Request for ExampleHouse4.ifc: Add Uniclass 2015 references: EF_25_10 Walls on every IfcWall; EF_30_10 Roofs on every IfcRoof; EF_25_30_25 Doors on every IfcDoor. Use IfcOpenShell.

First a look at what the model holds.

```python
import ifcopenshell

model = ifcopenshell.open("ExampleHouse4.ifc")
print(model.schema)
print("classifications:", [c.Name for c in model.by_type("IfcClassification")])
for ifc_class in ("IfcDoor", "IfcRoof", "IfcStair", "IfcWall", "IfcWindow"):
    print(ifc_class, len(model.by_type(ifc_class)))
```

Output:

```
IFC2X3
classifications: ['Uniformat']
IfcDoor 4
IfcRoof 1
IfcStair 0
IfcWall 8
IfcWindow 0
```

```python
import ifcopenshell
import ifcopenshell.api.classification

model = ifcopenshell.open("ExampleHouse4.ifc")

# IFC2X3 requires Source and Edition and has no link from the project to the system.
system = model.create_entity("IfcClassification", Source="NBS", Edition="2015", Name="Uniclass 2015")

codes = {
    "IfcWall": ("EF_25_10", "Walls"),
    "IfcRoof": ("EF_30_10", "Roofs"),
    "IfcDoor": ("EF_25_30_25", "Doors"),
}
for ifc_class, (code, name) in codes.items():
    products = model.by_type(ifc_class)
    ifcopenshell.api.classification.add_reference(
        model, products=products, classification=system, identification=code, name=name
    )
    print(code, len(products))

model.write("ExampleHouse4_v2.ifc")
```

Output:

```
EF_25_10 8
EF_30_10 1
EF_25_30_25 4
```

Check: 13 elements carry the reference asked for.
